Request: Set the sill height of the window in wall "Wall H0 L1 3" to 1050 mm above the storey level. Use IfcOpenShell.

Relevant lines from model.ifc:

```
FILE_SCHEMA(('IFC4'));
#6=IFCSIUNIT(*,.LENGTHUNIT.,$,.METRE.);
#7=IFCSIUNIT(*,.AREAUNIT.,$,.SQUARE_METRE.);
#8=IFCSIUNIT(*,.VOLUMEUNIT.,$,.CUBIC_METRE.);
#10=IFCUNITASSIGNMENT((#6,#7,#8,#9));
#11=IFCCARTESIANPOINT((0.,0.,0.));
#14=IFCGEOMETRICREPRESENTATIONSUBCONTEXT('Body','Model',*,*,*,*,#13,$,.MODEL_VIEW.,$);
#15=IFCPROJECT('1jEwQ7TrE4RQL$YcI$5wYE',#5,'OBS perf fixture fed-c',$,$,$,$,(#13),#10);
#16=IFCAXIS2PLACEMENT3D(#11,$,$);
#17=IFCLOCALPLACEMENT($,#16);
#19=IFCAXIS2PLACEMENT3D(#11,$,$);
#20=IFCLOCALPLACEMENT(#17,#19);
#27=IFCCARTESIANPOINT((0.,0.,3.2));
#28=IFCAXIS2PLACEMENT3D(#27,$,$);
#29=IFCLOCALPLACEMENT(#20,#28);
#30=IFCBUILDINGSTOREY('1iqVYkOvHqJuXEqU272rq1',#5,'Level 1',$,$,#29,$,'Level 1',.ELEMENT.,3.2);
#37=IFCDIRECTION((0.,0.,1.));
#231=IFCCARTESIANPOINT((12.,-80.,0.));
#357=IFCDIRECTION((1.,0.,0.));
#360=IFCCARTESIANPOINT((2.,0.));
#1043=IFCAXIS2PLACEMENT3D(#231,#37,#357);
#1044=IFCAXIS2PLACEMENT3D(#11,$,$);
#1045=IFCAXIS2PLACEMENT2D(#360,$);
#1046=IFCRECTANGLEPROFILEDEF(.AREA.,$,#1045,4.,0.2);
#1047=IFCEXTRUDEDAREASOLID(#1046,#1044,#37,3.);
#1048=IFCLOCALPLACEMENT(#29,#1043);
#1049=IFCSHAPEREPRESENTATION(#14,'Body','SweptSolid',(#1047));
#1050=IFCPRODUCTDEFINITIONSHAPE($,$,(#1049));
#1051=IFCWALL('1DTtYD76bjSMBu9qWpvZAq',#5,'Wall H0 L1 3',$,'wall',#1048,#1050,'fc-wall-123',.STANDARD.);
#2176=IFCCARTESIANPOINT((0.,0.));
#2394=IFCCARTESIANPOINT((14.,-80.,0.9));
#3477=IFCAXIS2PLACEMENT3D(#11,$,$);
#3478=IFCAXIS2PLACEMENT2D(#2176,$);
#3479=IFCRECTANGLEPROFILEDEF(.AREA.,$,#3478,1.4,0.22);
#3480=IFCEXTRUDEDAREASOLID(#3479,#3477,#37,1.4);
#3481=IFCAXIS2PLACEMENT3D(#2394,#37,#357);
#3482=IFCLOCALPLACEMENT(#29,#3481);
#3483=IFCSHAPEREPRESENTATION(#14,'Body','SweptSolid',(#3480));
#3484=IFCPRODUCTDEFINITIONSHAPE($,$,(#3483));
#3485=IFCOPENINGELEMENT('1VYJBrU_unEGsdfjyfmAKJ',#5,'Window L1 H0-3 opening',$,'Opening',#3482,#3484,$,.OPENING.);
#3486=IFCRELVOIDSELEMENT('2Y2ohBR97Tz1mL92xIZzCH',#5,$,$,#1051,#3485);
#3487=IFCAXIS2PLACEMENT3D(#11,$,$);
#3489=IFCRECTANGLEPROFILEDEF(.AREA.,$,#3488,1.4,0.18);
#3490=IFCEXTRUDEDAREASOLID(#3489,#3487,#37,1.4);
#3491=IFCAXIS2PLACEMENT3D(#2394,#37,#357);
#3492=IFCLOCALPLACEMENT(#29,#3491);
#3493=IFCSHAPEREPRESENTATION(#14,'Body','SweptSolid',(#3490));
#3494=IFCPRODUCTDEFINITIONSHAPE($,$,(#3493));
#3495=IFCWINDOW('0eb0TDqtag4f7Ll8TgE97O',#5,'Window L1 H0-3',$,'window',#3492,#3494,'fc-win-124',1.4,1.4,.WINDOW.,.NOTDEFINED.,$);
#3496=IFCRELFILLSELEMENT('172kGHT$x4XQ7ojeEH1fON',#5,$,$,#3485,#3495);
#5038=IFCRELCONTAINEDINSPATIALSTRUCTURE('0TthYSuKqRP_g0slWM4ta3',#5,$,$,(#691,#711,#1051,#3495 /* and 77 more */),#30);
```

```python
import numpy as np
import ifcopenshell
import ifcopenshell.api.geometry
import ifcopenshell.geom
import ifcopenshell.util.element
import ifcopenshell.util.placement
import ifcopenshell.util.shape
import ifcopenshell.util.unit

model = ifcopenshell.open("model.ifc")
unit_scale = ifcopenshell.util.unit.calculate_unit_scale(model)

window = model.by_id(3495)
opening = window.FillsVoids[0].RelatingOpeningElement
storey = ifcopenshell.util.element.get_container(window, ifc_class="IfcBuildingStorey")
level = ifcopenshell.util.placement.get_local_placement(storey.ObjectPlacement)[2, 3]

# The opening's origin need not be at the sill, so measure its lowest point.
shape = ifcopenshell.geom.create_shape(ifcopenshell.geom.settings(), opening)
bottom = ifcopenshell.util.shape.get_shape_bottom_elevation(shape, shape.geometry) / unit_scale
dz = level + 1.05 / unit_scale - bottom

shift = np.array([0.0, 0.0, dz])
# The window is not placed relative to its opening, so move both.
for product in (opening, window):
    matrix = ifcopenshell.util.placement.get_local_placement(product.ObjectPlacement)
    matrix[:3, 3] += shift
    ifcopenshell.api.geometry.edit_object_placement(model, product=product, matrix=matrix, is_si=False)

print(f"moved by {dz * unit_scale:+.3f} m")

model.write("model_v2.ifc")
```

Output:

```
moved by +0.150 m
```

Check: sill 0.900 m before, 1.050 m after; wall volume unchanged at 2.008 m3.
